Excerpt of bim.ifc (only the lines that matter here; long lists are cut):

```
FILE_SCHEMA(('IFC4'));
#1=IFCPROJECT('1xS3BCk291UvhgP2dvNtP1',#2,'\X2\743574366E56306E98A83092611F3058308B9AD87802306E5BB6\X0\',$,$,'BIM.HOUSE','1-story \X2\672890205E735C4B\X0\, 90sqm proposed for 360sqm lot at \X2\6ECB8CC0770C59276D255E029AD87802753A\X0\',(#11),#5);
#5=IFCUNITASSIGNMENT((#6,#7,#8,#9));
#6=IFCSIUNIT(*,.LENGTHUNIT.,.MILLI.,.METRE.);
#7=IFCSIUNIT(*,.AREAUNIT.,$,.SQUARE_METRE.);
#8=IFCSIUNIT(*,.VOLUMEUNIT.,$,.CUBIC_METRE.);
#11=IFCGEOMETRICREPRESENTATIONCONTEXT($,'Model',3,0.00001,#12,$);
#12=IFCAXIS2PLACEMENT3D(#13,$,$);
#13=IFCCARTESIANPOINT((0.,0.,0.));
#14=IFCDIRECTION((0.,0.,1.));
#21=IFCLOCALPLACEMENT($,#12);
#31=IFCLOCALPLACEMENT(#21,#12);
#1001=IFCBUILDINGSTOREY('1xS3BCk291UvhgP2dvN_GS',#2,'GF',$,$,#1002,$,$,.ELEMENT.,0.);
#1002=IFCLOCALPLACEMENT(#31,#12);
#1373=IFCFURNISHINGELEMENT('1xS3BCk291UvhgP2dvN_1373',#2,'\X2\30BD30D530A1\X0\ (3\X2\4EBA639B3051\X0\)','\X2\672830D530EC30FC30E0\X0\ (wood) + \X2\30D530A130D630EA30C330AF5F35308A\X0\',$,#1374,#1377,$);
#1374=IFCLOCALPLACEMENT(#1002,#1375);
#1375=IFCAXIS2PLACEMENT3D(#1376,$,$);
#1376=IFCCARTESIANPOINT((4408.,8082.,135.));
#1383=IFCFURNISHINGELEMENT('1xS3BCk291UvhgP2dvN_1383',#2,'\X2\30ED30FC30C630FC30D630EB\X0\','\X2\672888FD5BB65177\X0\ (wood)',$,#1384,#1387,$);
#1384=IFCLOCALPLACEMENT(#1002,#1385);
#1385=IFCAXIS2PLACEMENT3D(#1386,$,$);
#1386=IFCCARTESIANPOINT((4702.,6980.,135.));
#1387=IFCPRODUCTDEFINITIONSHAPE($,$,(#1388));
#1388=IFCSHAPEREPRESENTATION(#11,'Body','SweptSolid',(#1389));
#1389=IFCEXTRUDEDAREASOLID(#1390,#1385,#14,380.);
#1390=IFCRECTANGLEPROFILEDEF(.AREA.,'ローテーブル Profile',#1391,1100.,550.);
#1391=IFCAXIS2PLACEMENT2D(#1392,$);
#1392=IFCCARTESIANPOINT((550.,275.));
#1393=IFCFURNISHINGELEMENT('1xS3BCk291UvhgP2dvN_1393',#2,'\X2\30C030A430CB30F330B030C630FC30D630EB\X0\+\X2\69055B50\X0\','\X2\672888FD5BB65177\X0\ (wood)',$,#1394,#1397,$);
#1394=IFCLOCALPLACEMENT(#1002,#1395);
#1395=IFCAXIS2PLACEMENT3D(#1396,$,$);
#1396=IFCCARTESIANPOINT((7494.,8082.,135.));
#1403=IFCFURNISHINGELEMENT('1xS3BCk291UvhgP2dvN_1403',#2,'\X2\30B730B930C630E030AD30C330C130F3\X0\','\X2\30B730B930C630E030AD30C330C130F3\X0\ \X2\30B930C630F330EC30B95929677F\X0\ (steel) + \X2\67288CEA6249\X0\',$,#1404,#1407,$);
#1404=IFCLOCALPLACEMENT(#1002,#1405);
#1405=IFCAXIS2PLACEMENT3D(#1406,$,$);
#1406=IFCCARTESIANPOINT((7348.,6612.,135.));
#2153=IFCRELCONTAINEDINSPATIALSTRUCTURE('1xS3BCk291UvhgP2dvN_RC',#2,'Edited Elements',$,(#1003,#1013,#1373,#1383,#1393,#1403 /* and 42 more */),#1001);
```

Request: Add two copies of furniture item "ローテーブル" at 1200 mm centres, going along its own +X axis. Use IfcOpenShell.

```python
import ifcopenshell
import ifcopenshell.api.geometry
import ifcopenshell.api.root
import ifcopenshell.util.element
import ifcopenshell.util.placement
import ifcopenshell.util.unit

model = ifcopenshell.open("bim.ifc")
unit_scale = ifcopenshell.util.unit.calculate_unit_scale(model)


def reuse_history(source, copy):
    """copy_class also copies each property set's owner history, people and application; keep the originals."""
    for rel in copy.IsDefinedBy:
        if rel.is_a("IfcRelDefinesByProperties") and (history := rel.RelatingPropertyDefinition.OwnerHistory):
            rel.RelatingPropertyDefinition.OwnerHistory = source.OwnerHistory
            ifcopenshell.util.element.remove_deep2(model, history)


source = model.by_guid("1xS3BCk291UvhgP2dvN_1383")
base = ifcopenshell.util.placement.get_local_placement(source.ObjectPlacement)
step = base[:3, 0] * 1.2 / unit_scale

for i in range(1, 3):
    copy = ifcopenshell.api.root.copy_class(model, product=source)
    copy.Representation = ifcopenshell.util.element.copy_deep(
        model, source.Representation, exclude=["IfcGeometricRepresentationContext", "IfcRepresentationMap"]
    )
    reuse_history(source, copy)
    matrix = base.copy()
    matrix[:3, 3] += i * step
    print("added at", matrix[:3, 3].round(3) + 0.0)
    ifcopenshell.api.geometry.edit_object_placement(model, product=copy, matrix=matrix, is_si=False)

model.write("bim_v2.ifc")
```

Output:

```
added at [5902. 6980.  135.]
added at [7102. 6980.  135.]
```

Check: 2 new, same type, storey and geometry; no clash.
